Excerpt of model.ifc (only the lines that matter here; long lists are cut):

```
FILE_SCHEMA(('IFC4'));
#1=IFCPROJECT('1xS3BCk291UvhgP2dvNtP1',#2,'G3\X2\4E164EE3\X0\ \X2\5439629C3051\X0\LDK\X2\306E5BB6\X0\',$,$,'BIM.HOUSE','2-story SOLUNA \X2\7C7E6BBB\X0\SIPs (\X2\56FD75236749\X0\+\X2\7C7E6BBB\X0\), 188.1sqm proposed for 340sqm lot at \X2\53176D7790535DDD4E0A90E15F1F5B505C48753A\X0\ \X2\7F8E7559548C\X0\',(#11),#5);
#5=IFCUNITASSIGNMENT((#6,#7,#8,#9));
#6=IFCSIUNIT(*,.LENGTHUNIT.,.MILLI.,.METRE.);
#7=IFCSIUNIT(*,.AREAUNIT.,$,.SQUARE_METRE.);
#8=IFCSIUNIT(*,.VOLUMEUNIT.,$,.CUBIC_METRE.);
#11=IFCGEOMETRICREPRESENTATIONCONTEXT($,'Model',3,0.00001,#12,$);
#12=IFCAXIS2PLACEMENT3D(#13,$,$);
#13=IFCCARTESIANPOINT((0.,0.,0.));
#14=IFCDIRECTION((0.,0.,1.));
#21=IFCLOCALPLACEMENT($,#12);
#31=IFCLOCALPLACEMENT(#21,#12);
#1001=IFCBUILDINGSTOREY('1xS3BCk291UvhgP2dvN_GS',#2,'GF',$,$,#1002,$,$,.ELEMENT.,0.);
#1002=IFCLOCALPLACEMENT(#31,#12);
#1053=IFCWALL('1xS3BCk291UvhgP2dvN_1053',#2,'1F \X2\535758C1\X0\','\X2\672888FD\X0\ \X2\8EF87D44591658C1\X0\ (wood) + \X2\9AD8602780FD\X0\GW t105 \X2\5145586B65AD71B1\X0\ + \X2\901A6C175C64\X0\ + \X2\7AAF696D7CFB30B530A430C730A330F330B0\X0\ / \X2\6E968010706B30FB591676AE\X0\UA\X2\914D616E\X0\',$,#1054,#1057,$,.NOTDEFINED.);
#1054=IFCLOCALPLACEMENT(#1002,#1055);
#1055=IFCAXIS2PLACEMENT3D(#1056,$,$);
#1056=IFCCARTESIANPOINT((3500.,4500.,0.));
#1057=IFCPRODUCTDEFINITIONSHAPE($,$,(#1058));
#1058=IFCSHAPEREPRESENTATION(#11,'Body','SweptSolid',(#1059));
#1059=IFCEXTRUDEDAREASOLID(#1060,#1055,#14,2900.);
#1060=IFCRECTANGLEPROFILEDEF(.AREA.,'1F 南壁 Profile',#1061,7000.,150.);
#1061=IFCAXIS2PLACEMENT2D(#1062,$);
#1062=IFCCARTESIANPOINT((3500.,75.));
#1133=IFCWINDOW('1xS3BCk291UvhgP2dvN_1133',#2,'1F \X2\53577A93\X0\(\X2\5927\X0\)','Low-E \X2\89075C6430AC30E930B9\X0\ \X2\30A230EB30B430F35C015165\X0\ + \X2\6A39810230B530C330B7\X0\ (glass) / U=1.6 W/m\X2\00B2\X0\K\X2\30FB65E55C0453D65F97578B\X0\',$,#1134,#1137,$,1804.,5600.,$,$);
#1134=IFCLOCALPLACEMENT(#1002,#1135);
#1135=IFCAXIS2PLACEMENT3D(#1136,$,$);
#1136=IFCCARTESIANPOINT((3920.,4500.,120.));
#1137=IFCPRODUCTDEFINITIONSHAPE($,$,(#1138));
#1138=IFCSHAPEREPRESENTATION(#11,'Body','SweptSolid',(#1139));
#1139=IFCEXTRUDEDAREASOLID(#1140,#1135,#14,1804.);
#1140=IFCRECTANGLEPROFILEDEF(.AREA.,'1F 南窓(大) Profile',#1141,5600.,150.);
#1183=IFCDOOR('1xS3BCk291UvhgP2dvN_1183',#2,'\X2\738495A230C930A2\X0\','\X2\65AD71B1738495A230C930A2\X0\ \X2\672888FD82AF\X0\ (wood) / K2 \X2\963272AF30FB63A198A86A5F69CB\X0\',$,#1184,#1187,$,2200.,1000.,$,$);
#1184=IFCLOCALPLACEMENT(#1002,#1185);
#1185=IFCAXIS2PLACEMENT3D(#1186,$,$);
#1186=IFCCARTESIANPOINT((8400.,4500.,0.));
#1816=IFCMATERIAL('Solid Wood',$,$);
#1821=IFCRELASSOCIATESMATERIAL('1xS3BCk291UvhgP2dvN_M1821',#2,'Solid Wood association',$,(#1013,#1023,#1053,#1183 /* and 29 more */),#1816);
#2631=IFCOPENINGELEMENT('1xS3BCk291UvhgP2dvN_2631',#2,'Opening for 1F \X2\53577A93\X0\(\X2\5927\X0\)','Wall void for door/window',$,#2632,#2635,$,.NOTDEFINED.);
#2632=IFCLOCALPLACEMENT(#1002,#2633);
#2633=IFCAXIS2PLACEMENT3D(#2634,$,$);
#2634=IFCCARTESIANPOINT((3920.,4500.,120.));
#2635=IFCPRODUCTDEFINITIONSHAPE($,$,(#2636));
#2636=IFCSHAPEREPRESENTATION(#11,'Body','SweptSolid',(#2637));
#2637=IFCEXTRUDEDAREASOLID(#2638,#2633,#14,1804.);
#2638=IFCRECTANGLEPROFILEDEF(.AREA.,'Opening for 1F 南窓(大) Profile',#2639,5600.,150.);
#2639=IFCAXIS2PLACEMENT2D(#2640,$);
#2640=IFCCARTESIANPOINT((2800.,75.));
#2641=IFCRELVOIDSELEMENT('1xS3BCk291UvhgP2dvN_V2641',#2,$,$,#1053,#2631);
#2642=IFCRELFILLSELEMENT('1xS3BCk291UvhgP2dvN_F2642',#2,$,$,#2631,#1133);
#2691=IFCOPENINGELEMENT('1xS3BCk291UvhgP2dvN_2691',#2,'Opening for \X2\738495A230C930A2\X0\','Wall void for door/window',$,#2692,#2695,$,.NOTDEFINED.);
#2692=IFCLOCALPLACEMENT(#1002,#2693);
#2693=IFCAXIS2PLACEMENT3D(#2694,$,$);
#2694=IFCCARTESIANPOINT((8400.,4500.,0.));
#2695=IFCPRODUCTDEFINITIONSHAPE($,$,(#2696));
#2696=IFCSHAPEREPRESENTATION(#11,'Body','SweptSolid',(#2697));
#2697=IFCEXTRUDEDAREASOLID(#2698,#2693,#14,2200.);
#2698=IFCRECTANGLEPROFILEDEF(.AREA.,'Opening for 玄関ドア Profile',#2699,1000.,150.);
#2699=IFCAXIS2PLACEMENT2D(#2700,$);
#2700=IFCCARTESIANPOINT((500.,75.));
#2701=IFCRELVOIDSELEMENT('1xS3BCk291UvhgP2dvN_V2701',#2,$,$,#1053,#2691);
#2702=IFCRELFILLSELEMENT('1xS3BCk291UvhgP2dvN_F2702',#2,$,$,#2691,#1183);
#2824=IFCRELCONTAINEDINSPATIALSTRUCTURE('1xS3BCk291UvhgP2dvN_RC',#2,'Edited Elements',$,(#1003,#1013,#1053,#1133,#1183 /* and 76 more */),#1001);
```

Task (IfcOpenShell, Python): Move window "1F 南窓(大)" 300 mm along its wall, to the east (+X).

```python
import ifcopenshell
import ifcopenshell.api.geometry
import ifcopenshell.util.placement
import ifcopenshell.util.unit

model = ifcopenshell.open("model.ifc")
unit_scale = ifcopenshell.util.unit.calculate_unit_scale(model)

window = model.by_guid("1xS3BCk291UvhgP2dvN_1133")
opening = window.FillsVoids[0].RelatingOpeningElement
wall = opening.VoidsElements[0].RelatingBuildingElement

wall_matrix = ifcopenshell.util.placement.get_local_placement(wall.ObjectPlacement)
shift = wall_matrix[:3, 0] * 0.3 / unit_scale
before = ifcopenshell.util.placement.get_local_placement(window.ObjectPlacement)[:3, 3].copy()

# The window is not placed relative to its opening, so move both.
for product in (opening, window):
    matrix = ifcopenshell.util.placement.get_local_placement(product.ObjectPlacement)
    matrix[:3, 3] += shift
    ifcopenshell.api.geometry.edit_object_placement(model, product=product, matrix=matrix, is_si=False)

after = ifcopenshell.util.placement.get_local_placement(window.ObjectPlacement)[:3, 3]
print("window moved by", (after - before).round(3) + 0.0)

model.write("model_rev.ifc")
```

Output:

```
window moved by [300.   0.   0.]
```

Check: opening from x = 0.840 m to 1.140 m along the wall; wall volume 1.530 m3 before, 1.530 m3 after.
